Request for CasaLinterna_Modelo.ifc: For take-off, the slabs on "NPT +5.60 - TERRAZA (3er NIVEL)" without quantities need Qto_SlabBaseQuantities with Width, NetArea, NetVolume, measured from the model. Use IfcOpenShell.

First a look at what the model holds.

```python
import ifcopenshell
import ifcopenshell.util.element
import ifcopenshell.util.unit

model = ifcopenshell.open("CasaLinterna_Modelo.ifc")
print(model.schema)
for unit_type in ("LENGTHUNIT", "AREAUNIT", "VOLUMEUNIT"):
    print(unit_type, ifcopenshell.util.unit.calculate_unit_scale(model, unit_type))
storey = next(s for s in model.by_type("IfcBuildingStorey") if s.Name == "NPT +5.60 - TERRAZA (3er NIVEL)")
slabs = [e for e in ifcopenshell.util.element.get_decomposition(storey) if e.is_a("IfcSlab")]
for e in sorted(slabs, key=lambda e: e.id()):
    print(e.id(), e.is_a(), e.Name, list(ifcopenshell.util.element.get_psets(e, qtos_only=True)), sep=" | ")
```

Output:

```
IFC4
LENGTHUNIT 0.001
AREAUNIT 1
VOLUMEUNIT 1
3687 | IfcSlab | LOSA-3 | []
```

```python
import ifcopenshell
import ifcopenshell.api.pset
import ifcopenshell.geom
import ifcopenshell.util.element
import ifcopenshell.util.shape
import ifcopenshell.util.unit

model = ifcopenshell.open("CasaLinterna_Modelo.ifc")
unit_scale = ifcopenshell.util.unit.calculate_unit_scale(model)
area_scale = ifcopenshell.util.unit.calculate_unit_scale(model, "AREAUNIT")
volume_scale = ifcopenshell.util.unit.calculate_unit_scale(model, "VOLUMEUNIT")
settings = ifcopenshell.geom.settings()

storey = next(s for s in model.by_type("IfcBuildingStorey") if s.Name == "NPT +5.60 - TERRAZA (3er NIVEL)")
slabs = [e for e in ifcopenshell.util.element.get_decomposition(storey) if e.is_a("IfcSlab")]

for e in sorted(slabs, key=lambda e: e.id()):
    if ifcopenshell.util.element.get_psets(e, qtos_only=True, should_inherit=False):
        continue
    # Geometry comes back in metres, in the element's own axes.
    shape = ifcopenshell.geom.create_shape(settings, e)
    values = {
        "Width": ifcopenshell.util.shape.get_z(shape.geometry) / unit_scale,
        "NetArea": ifcopenshell.util.shape.get_footprint_area(shape.geometry) / area_scale,
        "NetVolume": ifcopenshell.util.shape.get_volume(shape.geometry) / volume_scale,
    }
    qto = ifcopenshell.api.pset.add_qto(model, product=e, name="Qto_SlabBaseQuantities")
    ifcopenshell.api.pset.edit_qto(model, qto=qto, properties=values)
    print(e.id(), {k: round(v, 3) for k, v in values.items()})

model.write("CasaLinterna_Modelo_v2.ifc")
```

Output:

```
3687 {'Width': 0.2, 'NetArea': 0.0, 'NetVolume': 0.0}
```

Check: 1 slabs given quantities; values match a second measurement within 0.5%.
